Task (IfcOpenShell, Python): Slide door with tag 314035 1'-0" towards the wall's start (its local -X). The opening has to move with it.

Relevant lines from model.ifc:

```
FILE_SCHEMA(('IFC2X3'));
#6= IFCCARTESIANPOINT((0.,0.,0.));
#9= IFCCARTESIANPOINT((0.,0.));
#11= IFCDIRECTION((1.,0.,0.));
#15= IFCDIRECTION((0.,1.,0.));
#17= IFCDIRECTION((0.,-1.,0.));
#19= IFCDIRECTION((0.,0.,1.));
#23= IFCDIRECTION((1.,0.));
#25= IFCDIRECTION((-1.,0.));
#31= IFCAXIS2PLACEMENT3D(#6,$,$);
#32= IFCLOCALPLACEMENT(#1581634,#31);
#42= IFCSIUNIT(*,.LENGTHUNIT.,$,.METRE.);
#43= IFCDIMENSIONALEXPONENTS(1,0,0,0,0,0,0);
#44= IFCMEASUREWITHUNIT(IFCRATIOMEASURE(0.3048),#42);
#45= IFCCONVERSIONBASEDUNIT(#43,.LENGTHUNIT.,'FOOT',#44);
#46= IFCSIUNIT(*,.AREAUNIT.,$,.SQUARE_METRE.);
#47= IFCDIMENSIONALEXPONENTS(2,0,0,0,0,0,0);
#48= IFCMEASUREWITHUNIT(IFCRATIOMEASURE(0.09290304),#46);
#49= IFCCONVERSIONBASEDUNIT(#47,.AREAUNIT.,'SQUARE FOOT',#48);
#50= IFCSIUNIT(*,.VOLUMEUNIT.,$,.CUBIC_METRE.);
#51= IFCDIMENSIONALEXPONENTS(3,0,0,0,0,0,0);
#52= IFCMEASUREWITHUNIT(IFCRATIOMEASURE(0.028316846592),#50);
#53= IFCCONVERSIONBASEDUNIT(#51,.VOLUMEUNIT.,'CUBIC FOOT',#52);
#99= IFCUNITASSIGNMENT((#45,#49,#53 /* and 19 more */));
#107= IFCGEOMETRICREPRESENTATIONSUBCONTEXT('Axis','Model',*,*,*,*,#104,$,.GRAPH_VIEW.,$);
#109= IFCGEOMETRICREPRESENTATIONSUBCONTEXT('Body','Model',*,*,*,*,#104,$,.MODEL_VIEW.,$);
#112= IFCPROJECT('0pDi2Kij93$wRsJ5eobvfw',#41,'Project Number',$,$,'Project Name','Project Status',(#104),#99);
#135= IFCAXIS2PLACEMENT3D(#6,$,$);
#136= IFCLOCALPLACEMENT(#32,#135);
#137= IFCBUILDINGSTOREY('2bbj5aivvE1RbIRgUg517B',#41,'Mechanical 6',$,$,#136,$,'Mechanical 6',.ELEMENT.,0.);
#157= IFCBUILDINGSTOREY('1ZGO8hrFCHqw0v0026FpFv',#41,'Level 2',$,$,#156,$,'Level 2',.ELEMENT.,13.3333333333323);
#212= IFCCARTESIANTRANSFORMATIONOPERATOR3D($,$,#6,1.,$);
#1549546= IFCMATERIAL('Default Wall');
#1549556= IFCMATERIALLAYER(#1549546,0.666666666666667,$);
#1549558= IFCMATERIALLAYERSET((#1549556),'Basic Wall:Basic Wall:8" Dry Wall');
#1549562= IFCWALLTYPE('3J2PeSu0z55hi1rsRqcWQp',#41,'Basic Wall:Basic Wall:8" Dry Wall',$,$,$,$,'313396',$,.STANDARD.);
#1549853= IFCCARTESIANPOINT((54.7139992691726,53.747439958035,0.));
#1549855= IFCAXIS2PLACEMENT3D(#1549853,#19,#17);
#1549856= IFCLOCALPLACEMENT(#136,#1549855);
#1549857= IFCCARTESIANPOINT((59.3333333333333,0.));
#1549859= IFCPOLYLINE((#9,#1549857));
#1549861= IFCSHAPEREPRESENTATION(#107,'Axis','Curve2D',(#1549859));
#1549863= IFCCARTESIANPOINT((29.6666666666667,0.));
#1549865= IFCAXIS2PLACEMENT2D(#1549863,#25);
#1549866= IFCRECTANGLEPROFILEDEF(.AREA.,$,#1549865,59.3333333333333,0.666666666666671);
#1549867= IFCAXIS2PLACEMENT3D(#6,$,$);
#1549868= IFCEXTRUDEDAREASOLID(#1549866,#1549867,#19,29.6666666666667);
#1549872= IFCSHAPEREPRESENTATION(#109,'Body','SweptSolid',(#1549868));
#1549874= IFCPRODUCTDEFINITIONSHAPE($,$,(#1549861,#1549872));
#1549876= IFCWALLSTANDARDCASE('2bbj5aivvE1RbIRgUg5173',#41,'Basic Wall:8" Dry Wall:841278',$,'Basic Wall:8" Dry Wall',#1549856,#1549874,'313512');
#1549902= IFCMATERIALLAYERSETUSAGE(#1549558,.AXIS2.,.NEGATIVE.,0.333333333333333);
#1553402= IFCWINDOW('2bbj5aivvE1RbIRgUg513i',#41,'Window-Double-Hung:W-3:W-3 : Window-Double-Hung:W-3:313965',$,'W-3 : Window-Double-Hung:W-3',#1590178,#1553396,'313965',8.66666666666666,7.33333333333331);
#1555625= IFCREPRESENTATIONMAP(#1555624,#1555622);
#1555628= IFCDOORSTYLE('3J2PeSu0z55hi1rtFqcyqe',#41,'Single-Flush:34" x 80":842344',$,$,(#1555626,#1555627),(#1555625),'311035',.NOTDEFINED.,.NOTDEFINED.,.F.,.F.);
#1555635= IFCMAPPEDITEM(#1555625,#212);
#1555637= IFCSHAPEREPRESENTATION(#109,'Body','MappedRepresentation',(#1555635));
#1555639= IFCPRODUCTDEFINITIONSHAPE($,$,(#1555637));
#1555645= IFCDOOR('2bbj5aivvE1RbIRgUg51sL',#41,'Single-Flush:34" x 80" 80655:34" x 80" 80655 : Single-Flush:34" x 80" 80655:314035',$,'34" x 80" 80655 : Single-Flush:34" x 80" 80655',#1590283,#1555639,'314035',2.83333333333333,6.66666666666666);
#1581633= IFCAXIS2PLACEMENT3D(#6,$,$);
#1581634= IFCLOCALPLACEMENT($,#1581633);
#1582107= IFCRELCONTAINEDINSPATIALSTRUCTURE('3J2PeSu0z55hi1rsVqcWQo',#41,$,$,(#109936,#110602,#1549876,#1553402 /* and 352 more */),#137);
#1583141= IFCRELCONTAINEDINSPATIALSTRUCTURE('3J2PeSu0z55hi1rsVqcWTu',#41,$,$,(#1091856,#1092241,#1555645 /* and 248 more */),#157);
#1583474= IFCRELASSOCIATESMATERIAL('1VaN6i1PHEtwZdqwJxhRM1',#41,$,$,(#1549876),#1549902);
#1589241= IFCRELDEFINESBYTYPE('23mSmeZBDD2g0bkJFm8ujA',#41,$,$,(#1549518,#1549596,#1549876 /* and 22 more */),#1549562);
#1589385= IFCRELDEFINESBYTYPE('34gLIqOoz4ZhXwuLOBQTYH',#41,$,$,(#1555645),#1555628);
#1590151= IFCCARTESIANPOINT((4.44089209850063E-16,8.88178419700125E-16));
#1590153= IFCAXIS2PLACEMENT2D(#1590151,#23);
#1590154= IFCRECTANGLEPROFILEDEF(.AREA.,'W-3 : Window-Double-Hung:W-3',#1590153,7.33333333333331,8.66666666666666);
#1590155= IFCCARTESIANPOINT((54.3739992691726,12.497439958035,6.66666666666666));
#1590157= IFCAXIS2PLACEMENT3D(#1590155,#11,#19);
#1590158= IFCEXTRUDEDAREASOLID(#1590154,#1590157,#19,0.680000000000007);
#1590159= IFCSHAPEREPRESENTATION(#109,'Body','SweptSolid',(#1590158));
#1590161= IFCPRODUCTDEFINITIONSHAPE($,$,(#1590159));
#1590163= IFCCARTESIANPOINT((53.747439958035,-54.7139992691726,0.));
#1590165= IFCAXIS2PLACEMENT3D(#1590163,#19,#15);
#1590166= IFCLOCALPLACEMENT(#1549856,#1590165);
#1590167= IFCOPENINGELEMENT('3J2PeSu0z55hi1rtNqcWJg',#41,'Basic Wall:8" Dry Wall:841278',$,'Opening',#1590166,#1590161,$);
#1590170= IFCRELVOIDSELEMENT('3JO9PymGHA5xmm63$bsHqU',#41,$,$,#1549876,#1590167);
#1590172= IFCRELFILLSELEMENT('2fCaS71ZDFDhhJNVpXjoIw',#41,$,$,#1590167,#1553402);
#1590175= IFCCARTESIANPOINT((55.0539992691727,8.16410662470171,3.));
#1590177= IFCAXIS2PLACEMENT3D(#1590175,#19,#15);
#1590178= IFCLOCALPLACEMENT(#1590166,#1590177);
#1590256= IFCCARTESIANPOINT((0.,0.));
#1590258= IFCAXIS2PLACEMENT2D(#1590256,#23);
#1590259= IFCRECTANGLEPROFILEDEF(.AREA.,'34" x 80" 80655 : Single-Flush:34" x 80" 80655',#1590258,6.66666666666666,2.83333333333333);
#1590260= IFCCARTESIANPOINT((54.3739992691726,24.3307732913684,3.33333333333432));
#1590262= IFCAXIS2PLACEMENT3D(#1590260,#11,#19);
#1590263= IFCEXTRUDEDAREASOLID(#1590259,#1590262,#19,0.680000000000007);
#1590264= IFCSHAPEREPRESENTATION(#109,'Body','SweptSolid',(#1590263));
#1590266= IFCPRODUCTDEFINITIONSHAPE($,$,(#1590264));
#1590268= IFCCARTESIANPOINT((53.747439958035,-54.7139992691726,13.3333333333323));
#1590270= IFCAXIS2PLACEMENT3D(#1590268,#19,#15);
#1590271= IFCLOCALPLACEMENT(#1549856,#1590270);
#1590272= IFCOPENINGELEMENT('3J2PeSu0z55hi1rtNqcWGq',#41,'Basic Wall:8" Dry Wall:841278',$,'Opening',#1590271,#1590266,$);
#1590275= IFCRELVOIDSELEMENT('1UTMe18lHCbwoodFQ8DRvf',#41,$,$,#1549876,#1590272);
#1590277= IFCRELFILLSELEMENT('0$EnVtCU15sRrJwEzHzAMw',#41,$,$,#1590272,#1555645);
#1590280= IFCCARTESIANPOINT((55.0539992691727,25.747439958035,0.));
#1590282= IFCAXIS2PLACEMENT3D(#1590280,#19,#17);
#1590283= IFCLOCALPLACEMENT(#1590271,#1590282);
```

```python
import ifcopenshell
import ifcopenshell.api.geometry
import ifcopenshell.util.placement
import ifcopenshell.util.unit

model = ifcopenshell.open("model.ifc")
unit_scale = ifcopenshell.util.unit.calculate_unit_scale(model)

door = model.by_guid("2bbj5aivvE1RbIRgUg51sL")
opening = door.FillsVoids[0].RelatingOpeningElement
wall = opening.VoidsElements[0].RelatingBuildingElement

wall_matrix = ifcopenshell.util.placement.get_local_placement(wall.ObjectPlacement)
shift = wall_matrix[:3, 0] * -12 * 0.0254 / unit_scale
before = ifcopenshell.util.placement.get_local_placement(door.ObjectPlacement)[:3, 3].copy()

# The door is placed relative to its opening, so it follows when the opening moves.
matrix = ifcopenshell.util.placement.get_local_placement(opening.ObjectPlacement)
matrix[:3, 3] += shift
ifcopenshell.api.geometry.edit_object_placement(
    model, product=opening, matrix=matrix, is_si=False, should_transform_children=True
)

after = ifcopenshell.util.placement.get_local_placement(door.ObjectPlacement)[:3, 3]
print("door moved by", (after - before).round(3) + 0.0)

model.write("model_v2.ifc")
```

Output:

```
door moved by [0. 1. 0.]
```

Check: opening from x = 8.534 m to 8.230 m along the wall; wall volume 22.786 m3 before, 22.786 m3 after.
